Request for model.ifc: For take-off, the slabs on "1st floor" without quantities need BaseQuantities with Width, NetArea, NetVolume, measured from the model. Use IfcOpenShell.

First a look at what the model holds.

```python
import ifcopenshell
import ifcopenshell.util.element
import ifcopenshell.util.unit

model = ifcopenshell.open("model.ifc")
print(model.schema)
for unit_type in ("LENGTHUNIT", "AREAUNIT", "VOLUMEUNIT"):
    print(unit_type, ifcopenshell.util.unit.calculate_unit_scale(model, unit_type))
storey = next(s for s in model.by_type("IfcBuildingStorey") if s.Name == "1st floor")
slabs = [e for e in ifcopenshell.util.element.get_decomposition(storey) if e.is_a("IfcSlab")]
for e in sorted(slabs, key=lambda e: e.id()):
    print(e.id(), e.is_a(), e.Name, list(ifcopenshell.util.element.get_psets(e, qtos_only=True)), sep=" | ")
```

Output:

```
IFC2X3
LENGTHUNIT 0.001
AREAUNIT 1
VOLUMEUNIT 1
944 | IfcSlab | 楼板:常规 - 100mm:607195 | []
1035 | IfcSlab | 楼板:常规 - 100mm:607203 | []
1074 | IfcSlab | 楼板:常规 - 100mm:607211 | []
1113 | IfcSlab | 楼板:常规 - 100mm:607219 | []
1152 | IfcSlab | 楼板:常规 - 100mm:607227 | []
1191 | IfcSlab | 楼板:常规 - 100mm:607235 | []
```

```python
import ifcopenshell
import ifcopenshell.api.pset
import ifcopenshell.geom
import ifcopenshell.util.element
import ifcopenshell.util.shape
import ifcopenshell.util.unit

model = ifcopenshell.open("model.ifc")
unit_scale = ifcopenshell.util.unit.calculate_unit_scale(model)
area_scale = ifcopenshell.util.unit.calculate_unit_scale(model, "AREAUNIT")
volume_scale = ifcopenshell.util.unit.calculate_unit_scale(model, "VOLUMEUNIT")
settings = ifcopenshell.geom.settings()

storey = next(s for s in model.by_type("IfcBuildingStorey") if s.Name == "1st floor")
slabs = [e for e in ifcopenshell.util.element.get_decomposition(storey) if e.is_a("IfcSlab")]

for e in sorted(slabs, key=lambda e: e.id()):
    if ifcopenshell.util.element.get_psets(e, qtos_only=True, should_inherit=False):
        continue
    # Geometry comes back in metres, in the element's own axes.
    shape = ifcopenshell.geom.create_shape(settings, e)
    values = {
        "Width": ifcopenshell.util.shape.get_z(shape.geometry) / unit_scale,
        "NetArea": ifcopenshell.util.shape.get_footprint_area(shape.geometry) / area_scale,
        "NetVolume": ifcopenshell.util.shape.get_volume(shape.geometry) / volume_scale,
    }
    qto = ifcopenshell.api.pset.add_qto(model, product=e, name="BaseQuantities")
    ifcopenshell.api.pset.edit_qto(model, qto=qto, properties=values)
    print(e.id(), {k: round(v, 3) for k, v in values.items()})

model.write("model_edited.ifc")
```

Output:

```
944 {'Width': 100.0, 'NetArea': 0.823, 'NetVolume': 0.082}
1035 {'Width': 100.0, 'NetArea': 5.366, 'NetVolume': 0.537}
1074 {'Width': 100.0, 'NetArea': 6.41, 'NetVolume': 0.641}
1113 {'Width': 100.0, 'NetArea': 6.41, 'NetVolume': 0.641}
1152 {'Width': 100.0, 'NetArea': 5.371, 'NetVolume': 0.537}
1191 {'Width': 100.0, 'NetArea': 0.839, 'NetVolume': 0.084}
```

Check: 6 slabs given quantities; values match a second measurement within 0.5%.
